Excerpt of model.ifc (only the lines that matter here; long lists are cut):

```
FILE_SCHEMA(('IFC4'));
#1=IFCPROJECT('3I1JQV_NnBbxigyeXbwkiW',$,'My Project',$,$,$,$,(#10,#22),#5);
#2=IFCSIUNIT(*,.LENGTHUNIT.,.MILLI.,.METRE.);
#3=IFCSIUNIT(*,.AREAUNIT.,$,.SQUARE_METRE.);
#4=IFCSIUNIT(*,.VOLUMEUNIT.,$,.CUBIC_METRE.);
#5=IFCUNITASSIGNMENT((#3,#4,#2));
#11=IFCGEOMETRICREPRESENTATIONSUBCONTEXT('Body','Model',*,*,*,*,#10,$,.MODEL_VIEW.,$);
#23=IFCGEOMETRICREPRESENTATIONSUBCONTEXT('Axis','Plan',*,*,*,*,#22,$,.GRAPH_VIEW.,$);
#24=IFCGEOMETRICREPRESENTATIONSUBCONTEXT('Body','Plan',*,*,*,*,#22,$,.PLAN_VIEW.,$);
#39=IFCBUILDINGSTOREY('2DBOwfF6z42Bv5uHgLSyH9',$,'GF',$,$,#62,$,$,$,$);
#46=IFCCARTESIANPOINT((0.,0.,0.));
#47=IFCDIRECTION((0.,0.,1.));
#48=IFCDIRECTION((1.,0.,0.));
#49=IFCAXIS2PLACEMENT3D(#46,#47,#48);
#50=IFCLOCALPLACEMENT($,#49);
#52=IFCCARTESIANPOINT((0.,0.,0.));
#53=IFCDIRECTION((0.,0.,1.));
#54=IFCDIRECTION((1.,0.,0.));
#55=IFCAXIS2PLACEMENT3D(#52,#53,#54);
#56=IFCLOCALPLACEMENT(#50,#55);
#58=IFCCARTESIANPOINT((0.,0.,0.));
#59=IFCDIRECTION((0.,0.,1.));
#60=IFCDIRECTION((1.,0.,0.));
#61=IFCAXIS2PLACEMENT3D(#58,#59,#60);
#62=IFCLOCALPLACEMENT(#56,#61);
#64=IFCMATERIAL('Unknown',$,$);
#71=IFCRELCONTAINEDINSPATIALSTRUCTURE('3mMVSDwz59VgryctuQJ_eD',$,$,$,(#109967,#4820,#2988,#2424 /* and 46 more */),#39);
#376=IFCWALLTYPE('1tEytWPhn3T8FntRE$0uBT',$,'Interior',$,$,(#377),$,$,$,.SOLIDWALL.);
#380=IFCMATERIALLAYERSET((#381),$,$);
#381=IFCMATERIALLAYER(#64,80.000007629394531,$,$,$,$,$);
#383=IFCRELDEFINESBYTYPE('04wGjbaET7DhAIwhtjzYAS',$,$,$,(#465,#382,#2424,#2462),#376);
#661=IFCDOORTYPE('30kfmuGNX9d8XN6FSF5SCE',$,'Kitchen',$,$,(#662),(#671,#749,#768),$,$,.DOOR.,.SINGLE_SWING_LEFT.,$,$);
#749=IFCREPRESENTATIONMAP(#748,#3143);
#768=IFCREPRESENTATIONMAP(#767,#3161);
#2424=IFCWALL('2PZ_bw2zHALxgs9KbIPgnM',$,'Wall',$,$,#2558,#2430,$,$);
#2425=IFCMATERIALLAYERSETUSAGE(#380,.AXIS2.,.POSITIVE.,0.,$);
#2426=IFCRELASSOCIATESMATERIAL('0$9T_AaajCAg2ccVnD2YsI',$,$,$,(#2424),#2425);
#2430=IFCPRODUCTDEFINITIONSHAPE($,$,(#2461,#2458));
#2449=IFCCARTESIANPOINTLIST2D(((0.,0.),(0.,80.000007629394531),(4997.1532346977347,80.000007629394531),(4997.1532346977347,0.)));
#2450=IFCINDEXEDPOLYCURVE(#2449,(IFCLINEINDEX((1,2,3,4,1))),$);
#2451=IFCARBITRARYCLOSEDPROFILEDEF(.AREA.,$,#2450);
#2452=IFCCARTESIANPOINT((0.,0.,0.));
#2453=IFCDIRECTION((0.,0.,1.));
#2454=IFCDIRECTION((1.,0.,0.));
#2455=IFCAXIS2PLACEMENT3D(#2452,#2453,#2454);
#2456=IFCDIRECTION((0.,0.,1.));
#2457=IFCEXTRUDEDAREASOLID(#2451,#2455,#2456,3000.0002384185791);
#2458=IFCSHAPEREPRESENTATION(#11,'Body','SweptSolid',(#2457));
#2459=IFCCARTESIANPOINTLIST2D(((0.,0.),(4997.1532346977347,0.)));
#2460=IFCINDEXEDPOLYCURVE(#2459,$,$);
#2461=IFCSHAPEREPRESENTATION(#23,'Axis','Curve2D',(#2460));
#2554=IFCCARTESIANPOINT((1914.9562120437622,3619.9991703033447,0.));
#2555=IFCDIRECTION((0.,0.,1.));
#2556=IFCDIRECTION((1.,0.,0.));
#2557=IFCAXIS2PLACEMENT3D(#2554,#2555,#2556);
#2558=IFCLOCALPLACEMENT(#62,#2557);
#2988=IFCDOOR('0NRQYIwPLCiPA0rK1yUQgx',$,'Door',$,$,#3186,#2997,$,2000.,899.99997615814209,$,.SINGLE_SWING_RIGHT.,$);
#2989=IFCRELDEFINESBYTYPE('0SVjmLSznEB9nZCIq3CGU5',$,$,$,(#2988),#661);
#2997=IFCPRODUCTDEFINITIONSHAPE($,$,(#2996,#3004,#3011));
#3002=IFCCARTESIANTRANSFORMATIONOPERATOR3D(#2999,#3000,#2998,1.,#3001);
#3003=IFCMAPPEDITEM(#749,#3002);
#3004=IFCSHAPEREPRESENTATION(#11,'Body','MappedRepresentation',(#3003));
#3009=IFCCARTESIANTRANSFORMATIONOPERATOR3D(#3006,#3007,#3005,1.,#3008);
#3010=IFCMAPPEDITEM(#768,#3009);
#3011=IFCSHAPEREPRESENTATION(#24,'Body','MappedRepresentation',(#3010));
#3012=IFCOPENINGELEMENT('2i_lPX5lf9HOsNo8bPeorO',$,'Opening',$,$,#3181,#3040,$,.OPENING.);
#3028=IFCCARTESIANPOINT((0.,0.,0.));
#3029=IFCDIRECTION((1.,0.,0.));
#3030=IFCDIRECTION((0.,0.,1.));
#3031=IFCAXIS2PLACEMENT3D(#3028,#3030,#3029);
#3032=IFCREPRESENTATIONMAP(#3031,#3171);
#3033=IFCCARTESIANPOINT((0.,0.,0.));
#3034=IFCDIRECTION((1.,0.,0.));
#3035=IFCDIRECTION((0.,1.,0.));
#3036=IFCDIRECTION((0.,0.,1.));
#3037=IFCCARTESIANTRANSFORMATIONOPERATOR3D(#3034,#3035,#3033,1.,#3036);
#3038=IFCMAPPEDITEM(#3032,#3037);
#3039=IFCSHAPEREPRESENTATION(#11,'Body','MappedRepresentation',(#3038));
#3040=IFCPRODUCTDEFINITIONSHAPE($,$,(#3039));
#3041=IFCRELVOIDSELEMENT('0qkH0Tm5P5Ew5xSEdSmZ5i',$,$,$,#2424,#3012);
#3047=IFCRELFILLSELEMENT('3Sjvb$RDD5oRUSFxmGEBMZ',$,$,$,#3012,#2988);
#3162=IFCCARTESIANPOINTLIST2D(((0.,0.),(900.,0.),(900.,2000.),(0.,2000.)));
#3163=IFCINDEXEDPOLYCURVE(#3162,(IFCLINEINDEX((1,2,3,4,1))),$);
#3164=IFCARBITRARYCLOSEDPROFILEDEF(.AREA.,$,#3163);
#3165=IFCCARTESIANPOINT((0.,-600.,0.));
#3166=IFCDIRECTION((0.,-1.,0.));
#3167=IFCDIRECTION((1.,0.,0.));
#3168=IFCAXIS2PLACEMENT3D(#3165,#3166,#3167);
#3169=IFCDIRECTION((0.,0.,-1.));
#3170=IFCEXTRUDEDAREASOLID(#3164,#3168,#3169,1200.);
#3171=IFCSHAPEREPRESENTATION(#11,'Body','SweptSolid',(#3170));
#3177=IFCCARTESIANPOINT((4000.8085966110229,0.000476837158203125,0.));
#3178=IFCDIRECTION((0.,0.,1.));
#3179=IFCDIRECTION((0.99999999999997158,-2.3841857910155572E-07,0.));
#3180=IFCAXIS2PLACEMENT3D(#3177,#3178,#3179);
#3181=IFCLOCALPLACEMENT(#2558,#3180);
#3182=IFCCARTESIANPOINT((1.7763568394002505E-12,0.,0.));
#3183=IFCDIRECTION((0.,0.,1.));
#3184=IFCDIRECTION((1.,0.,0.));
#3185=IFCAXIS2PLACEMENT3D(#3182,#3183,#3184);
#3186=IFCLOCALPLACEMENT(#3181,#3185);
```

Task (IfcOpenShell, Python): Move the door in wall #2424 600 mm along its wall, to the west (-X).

```python
import ifcopenshell
import ifcopenshell.api.geometry
import ifcopenshell.util.placement

model = ifcopenshell.open("model.ifc")

door = model.by_id(2988)
opening = door.FillsVoids[0].RelatingOpeningElement
wall = opening.VoidsElements[0].RelatingBuildingElement

wall_matrix = ifcopenshell.util.placement.get_local_placement(wall.ObjectPlacement)
shift = wall_matrix[:3, 0] * -600.0
before = ifcopenshell.util.placement.get_local_placement(door.ObjectPlacement)[:3, 3].copy()

# The door is placed relative to its opening, so it follows when the opening moves.
matrix = ifcopenshell.util.placement.get_local_placement(opening.ObjectPlacement)
matrix[:3, 3] += shift
ifcopenshell.api.geometry.edit_object_placement(
    model, product=opening, matrix=matrix, is_si=False, should_transform_children=True
)

after = ifcopenshell.util.placement.get_local_placement(door.ObjectPlacement)[:3, 3]
print("door moved by", (after - before).round(3) + 0.0)

model.write("model_rev.ifc")
```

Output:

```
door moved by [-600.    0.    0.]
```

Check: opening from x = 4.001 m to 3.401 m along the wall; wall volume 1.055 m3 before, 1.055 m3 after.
